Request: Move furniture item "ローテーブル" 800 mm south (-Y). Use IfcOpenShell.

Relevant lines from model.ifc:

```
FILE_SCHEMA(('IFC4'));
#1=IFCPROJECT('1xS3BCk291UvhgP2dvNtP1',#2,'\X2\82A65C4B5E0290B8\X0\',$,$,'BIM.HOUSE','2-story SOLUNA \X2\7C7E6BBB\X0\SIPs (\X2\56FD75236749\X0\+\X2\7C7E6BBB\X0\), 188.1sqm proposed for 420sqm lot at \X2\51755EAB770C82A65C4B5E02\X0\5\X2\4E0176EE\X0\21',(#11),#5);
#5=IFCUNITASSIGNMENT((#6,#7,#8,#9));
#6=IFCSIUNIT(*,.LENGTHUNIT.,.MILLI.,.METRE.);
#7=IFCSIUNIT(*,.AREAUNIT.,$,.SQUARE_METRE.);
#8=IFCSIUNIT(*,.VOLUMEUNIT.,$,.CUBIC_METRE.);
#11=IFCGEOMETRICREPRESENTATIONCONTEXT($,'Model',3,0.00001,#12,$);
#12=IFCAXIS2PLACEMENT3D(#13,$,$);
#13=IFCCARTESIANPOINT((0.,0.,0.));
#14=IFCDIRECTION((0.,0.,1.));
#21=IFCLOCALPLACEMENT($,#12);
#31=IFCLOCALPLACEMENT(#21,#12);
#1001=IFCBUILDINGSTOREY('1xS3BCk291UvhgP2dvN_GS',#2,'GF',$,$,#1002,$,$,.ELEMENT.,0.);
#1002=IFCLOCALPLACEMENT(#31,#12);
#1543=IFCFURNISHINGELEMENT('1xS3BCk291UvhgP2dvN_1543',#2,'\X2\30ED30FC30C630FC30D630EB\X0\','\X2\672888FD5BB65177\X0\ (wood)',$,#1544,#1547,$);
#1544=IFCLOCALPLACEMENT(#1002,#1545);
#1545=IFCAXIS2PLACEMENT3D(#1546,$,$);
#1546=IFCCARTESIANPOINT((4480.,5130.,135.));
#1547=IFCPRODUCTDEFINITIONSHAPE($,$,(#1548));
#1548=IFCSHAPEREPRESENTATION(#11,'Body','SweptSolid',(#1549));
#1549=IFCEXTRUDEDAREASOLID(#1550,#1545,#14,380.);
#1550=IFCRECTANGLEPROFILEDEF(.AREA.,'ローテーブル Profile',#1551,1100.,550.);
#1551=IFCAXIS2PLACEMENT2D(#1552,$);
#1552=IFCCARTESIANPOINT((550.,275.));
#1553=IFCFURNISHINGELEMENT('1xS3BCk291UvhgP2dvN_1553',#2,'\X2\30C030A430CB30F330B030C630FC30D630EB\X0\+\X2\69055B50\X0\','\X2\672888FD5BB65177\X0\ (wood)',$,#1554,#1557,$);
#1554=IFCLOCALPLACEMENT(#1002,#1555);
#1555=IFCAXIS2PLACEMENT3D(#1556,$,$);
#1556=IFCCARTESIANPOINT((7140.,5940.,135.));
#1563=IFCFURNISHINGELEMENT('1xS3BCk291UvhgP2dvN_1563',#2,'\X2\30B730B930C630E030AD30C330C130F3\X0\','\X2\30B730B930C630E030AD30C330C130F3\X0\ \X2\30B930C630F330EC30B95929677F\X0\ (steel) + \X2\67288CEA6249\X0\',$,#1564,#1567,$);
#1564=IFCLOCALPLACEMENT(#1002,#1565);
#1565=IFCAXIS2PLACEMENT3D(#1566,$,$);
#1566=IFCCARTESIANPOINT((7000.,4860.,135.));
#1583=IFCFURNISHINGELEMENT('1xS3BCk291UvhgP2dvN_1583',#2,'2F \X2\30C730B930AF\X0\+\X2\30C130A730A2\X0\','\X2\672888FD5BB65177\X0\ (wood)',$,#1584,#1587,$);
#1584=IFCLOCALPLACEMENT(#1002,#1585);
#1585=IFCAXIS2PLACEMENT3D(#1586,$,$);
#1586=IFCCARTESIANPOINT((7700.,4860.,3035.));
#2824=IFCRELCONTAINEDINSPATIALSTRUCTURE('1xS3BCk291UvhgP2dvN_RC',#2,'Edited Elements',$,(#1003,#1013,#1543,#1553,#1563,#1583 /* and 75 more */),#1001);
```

```python
import ifcopenshell
import ifcopenshell.api.geometry
import ifcopenshell.util.placement

model = ifcopenshell.open("model.ifc")

item = model.by_id(1543)
matrix = ifcopenshell.util.placement.get_local_placement(item.ObjectPlacement)
matrix[1, 3] -= 800.0
ifcopenshell.api.geometry.edit_object_placement(model, product=item, matrix=matrix, is_si=False)

print(ifcopenshell.util.placement.get_local_placement(item.ObjectPlacement).round(3) + 0.0)

model.write("model_updated.ifc")
```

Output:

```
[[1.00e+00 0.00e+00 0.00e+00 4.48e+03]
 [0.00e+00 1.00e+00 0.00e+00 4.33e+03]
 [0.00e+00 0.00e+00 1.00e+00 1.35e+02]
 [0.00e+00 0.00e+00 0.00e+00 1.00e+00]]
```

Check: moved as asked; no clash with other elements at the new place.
